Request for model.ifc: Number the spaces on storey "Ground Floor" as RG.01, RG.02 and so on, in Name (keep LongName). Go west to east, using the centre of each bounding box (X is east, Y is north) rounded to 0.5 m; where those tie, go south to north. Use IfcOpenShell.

First a look at what the model holds.

```python
import ifcopenshell
import ifcopenshell.util.element
import ifcopenshell.util.placement

model = ifcopenshell.open("model.ifc")
print(model.schema)
storey = next(s for s in model.by_type("IfcBuildingStorey") if s.Name == "Ground Floor")
spaces = [e for e in ifcopenshell.util.element.get_decomposition(storey) if e.is_a("IfcSpace")]
for e in sorted(spaces, key=lambda e: e.id()):
    origin = ifcopenshell.util.placement.get_local_placement(e.ObjectPlacement)[:3, 3]
    print(e.id(), e.Name, e.LongName, origin.round(2) + 0.0, sep=" | ")
```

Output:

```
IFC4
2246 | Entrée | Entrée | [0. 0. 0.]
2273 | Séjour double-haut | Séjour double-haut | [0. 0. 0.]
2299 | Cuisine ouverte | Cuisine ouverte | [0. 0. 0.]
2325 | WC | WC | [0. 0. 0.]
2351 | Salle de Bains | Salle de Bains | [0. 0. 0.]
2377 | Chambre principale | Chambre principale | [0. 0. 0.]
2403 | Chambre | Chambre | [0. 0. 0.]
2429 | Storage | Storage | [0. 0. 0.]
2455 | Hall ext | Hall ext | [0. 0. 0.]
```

```python
import ifcopenshell
import ifcopenshell.geom
import ifcopenshell.util.element
import ifcopenshell.util.shape

model = ifcopenshell.open("model.ifc")
settings = ifcopenshell.geom.settings()
settings.set("use-world-coords", True)


def centre(element):
    shape = ifcopenshell.geom.create_shape(settings, element)
    return ifcopenshell.util.shape.get_bbox_centroid(shape.geometry)


storey = next(s for s in model.by_type("IfcBuildingStorey") if s.Name == "Ground Floor")
spaces = [e for e in ifcopenshell.util.element.get_decomposition(storey) if e.is_a("IfcSpace")]

# Insertion points can sit at a corner or the storey origin, so sort by the geometry (in metres).
centres = {e: centre(e) for e in spaces}
spaces.sort(key=lambda e: (round(centres[e][0] / 0.5), centres[e][1]))

for i, e in enumerate(spaces, start=1):
    number = f"RG.{i:02d}"
    e.Name = number
    print(e.id(), number)

model.write("model_v2.ifc")
```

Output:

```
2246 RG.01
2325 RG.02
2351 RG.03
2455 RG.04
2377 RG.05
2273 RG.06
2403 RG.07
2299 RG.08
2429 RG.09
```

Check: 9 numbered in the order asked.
